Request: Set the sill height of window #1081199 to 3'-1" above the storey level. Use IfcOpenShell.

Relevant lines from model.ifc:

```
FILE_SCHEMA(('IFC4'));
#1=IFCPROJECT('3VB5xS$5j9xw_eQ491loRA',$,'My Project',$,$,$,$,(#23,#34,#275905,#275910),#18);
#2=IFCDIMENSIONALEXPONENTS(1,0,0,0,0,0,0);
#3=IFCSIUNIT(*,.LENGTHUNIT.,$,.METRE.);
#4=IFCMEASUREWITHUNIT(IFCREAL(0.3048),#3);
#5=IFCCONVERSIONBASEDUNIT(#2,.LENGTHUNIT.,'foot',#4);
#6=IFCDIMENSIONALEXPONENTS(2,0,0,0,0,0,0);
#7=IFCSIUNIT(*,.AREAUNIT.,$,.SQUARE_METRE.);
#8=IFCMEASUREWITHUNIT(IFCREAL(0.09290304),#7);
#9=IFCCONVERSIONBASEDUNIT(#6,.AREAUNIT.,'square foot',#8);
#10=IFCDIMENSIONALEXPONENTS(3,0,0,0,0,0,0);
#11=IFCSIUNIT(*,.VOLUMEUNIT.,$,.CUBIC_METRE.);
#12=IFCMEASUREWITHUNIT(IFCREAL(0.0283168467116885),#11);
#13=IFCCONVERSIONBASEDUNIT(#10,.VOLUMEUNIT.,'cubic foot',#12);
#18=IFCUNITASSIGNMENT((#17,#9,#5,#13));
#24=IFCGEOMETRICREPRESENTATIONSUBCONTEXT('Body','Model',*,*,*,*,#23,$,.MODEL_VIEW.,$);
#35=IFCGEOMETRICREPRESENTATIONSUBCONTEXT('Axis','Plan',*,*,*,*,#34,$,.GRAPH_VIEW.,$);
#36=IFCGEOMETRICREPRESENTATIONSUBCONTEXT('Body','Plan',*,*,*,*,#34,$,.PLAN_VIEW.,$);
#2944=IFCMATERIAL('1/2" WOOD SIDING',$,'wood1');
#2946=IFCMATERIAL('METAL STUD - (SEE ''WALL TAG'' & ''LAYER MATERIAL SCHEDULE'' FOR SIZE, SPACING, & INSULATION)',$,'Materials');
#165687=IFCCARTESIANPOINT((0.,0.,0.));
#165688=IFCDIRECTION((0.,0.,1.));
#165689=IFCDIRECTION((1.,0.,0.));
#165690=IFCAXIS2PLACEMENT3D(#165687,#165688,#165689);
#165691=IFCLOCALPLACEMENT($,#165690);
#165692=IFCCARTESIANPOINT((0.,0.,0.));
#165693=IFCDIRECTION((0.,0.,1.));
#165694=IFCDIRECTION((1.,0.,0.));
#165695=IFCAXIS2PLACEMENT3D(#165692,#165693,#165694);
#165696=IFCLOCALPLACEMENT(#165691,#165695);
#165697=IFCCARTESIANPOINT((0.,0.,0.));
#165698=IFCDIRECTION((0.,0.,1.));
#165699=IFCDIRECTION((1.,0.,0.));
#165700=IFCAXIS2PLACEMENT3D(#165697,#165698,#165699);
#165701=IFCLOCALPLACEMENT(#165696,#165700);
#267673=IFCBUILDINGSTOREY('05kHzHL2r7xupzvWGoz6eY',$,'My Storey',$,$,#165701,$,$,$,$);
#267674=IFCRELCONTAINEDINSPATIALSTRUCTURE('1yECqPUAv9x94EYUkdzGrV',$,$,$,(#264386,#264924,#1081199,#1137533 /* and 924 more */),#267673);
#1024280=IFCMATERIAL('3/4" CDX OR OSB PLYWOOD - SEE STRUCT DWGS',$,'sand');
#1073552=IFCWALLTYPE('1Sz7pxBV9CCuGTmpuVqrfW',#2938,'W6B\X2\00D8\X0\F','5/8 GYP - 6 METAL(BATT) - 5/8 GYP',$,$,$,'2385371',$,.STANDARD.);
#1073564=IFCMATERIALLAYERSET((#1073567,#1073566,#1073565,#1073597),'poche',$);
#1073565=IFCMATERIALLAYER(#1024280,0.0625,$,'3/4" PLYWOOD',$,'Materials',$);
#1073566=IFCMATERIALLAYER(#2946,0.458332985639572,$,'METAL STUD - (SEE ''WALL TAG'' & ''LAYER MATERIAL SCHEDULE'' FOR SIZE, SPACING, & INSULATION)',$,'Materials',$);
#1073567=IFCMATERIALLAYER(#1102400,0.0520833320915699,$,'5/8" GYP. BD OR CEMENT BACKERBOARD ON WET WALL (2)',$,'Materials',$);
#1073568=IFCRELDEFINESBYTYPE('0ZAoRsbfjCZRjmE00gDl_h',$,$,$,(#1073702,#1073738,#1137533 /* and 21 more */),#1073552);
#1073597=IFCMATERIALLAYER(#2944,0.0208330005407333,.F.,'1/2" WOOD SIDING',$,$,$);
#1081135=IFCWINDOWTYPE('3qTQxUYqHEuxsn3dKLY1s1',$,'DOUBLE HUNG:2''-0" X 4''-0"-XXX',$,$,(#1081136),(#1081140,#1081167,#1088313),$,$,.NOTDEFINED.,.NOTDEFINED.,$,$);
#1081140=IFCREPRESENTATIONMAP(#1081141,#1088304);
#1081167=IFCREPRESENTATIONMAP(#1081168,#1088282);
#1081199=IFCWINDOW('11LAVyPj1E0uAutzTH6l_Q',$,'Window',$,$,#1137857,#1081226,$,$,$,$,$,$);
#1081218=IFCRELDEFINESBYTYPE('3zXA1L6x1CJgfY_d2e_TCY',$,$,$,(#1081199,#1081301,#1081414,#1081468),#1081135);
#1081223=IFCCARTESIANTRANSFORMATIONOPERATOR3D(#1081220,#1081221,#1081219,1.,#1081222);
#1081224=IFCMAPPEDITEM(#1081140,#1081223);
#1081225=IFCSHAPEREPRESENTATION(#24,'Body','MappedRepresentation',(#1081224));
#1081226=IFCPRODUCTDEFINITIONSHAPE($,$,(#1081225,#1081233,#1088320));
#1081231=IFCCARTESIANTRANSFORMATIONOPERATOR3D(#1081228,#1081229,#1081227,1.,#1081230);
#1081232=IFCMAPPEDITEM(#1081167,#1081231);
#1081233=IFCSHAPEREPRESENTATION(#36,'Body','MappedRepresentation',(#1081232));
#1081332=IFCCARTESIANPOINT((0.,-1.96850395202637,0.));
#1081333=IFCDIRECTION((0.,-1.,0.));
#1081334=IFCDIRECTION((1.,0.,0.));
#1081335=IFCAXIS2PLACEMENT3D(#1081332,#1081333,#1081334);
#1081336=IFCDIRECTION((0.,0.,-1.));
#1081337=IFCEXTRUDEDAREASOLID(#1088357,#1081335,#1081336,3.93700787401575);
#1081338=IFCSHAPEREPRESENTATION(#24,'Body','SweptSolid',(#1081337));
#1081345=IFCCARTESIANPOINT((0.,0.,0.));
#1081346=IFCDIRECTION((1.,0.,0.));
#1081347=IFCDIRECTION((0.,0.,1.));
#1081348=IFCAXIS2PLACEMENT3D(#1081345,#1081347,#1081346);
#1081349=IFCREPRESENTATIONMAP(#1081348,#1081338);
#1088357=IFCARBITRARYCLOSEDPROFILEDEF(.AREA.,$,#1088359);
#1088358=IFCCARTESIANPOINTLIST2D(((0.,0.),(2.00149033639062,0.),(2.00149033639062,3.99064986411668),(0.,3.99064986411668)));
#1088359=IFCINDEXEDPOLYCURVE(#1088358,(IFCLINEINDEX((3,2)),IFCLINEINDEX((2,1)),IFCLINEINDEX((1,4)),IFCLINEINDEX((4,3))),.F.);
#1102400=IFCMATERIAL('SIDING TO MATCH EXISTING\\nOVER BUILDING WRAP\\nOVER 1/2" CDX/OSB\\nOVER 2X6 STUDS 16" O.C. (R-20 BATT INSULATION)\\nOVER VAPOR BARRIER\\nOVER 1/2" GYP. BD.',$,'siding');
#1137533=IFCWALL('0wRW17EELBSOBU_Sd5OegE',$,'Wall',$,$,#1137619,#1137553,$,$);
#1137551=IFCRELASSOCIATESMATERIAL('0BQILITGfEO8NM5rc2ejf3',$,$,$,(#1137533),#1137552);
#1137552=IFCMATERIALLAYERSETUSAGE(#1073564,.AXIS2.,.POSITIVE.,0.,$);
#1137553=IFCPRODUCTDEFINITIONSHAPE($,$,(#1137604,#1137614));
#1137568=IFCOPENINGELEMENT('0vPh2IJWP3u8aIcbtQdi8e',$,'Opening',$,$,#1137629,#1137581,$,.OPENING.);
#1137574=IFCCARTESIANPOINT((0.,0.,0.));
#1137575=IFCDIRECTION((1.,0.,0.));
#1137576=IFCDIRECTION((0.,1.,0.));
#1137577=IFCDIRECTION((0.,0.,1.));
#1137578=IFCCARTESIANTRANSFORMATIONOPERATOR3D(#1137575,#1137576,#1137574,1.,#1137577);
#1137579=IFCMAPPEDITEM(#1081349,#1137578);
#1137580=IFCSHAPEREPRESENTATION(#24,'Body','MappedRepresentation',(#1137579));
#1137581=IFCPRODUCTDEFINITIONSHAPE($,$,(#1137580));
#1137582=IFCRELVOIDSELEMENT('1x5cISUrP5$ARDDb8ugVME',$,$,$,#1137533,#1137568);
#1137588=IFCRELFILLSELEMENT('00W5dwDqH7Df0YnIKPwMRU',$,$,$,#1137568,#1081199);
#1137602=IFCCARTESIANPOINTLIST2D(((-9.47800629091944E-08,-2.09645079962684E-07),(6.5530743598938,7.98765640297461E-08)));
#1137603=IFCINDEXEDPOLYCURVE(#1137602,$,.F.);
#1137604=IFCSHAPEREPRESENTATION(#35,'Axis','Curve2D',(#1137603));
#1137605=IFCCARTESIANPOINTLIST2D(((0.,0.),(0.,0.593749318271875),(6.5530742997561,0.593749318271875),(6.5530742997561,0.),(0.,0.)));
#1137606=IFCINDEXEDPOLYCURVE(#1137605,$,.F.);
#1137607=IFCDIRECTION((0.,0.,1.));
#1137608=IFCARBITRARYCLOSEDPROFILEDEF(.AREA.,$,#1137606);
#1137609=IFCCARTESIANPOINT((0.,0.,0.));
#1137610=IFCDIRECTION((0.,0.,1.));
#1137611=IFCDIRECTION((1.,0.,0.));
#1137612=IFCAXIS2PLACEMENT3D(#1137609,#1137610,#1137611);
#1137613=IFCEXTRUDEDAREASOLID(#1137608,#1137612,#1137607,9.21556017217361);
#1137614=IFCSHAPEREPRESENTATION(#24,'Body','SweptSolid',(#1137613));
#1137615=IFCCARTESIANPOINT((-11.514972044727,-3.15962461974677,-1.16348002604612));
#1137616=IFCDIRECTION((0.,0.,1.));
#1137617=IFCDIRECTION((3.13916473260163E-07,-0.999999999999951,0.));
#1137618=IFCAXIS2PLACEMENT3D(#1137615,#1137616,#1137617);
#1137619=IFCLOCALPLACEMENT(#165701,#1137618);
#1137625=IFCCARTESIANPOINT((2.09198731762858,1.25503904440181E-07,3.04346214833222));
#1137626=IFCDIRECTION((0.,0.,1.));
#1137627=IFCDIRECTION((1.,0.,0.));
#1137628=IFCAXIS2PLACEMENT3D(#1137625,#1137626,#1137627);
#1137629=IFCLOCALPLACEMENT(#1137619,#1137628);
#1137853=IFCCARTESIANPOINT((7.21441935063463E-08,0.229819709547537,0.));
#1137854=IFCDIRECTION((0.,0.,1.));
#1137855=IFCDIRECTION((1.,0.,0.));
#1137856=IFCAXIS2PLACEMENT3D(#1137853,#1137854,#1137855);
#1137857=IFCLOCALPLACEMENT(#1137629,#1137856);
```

```python
import numpy as np
import ifcopenshell
import ifcopenshell.api.geometry
import ifcopenshell.geom
import ifcopenshell.util.element
import ifcopenshell.util.placement
import ifcopenshell.util.shape
import ifcopenshell.util.unit

model = ifcopenshell.open("model.ifc")
unit_scale = ifcopenshell.util.unit.calculate_unit_scale(model)

window = model.by_guid("11LAVyPj1E0uAutzTH6l_Q")
opening = window.FillsVoids[0].RelatingOpeningElement
storey = ifcopenshell.util.element.get_container(window, ifc_class="IfcBuildingStorey")
level = ifcopenshell.util.placement.get_local_placement(storey.ObjectPlacement)[2, 3]

# The opening's origin need not be at the sill, so measure its lowest point.
shape = ifcopenshell.geom.create_shape(ifcopenshell.geom.settings(), opening)
bottom = ifcopenshell.util.shape.get_shape_bottom_elevation(shape, shape.geometry) / unit_scale
dz = level + 37 * 0.0254 / unit_scale - bottom

shift = np.array([0.0, 0.0, dz])
# The window is placed relative to its opening, so it follows when the opening moves.
matrix = ifcopenshell.util.placement.get_local_placement(opening.ObjectPlacement)
matrix[:3, 3] += shift
ifcopenshell.api.geometry.edit_object_placement(
    model, product=opening, matrix=matrix, is_si=False, should_transform_children=True
)

print(f"moved by {dz * unit_scale:+.3f} m")

model.write("model-out.ifc")
```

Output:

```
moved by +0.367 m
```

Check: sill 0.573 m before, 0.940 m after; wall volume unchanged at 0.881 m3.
